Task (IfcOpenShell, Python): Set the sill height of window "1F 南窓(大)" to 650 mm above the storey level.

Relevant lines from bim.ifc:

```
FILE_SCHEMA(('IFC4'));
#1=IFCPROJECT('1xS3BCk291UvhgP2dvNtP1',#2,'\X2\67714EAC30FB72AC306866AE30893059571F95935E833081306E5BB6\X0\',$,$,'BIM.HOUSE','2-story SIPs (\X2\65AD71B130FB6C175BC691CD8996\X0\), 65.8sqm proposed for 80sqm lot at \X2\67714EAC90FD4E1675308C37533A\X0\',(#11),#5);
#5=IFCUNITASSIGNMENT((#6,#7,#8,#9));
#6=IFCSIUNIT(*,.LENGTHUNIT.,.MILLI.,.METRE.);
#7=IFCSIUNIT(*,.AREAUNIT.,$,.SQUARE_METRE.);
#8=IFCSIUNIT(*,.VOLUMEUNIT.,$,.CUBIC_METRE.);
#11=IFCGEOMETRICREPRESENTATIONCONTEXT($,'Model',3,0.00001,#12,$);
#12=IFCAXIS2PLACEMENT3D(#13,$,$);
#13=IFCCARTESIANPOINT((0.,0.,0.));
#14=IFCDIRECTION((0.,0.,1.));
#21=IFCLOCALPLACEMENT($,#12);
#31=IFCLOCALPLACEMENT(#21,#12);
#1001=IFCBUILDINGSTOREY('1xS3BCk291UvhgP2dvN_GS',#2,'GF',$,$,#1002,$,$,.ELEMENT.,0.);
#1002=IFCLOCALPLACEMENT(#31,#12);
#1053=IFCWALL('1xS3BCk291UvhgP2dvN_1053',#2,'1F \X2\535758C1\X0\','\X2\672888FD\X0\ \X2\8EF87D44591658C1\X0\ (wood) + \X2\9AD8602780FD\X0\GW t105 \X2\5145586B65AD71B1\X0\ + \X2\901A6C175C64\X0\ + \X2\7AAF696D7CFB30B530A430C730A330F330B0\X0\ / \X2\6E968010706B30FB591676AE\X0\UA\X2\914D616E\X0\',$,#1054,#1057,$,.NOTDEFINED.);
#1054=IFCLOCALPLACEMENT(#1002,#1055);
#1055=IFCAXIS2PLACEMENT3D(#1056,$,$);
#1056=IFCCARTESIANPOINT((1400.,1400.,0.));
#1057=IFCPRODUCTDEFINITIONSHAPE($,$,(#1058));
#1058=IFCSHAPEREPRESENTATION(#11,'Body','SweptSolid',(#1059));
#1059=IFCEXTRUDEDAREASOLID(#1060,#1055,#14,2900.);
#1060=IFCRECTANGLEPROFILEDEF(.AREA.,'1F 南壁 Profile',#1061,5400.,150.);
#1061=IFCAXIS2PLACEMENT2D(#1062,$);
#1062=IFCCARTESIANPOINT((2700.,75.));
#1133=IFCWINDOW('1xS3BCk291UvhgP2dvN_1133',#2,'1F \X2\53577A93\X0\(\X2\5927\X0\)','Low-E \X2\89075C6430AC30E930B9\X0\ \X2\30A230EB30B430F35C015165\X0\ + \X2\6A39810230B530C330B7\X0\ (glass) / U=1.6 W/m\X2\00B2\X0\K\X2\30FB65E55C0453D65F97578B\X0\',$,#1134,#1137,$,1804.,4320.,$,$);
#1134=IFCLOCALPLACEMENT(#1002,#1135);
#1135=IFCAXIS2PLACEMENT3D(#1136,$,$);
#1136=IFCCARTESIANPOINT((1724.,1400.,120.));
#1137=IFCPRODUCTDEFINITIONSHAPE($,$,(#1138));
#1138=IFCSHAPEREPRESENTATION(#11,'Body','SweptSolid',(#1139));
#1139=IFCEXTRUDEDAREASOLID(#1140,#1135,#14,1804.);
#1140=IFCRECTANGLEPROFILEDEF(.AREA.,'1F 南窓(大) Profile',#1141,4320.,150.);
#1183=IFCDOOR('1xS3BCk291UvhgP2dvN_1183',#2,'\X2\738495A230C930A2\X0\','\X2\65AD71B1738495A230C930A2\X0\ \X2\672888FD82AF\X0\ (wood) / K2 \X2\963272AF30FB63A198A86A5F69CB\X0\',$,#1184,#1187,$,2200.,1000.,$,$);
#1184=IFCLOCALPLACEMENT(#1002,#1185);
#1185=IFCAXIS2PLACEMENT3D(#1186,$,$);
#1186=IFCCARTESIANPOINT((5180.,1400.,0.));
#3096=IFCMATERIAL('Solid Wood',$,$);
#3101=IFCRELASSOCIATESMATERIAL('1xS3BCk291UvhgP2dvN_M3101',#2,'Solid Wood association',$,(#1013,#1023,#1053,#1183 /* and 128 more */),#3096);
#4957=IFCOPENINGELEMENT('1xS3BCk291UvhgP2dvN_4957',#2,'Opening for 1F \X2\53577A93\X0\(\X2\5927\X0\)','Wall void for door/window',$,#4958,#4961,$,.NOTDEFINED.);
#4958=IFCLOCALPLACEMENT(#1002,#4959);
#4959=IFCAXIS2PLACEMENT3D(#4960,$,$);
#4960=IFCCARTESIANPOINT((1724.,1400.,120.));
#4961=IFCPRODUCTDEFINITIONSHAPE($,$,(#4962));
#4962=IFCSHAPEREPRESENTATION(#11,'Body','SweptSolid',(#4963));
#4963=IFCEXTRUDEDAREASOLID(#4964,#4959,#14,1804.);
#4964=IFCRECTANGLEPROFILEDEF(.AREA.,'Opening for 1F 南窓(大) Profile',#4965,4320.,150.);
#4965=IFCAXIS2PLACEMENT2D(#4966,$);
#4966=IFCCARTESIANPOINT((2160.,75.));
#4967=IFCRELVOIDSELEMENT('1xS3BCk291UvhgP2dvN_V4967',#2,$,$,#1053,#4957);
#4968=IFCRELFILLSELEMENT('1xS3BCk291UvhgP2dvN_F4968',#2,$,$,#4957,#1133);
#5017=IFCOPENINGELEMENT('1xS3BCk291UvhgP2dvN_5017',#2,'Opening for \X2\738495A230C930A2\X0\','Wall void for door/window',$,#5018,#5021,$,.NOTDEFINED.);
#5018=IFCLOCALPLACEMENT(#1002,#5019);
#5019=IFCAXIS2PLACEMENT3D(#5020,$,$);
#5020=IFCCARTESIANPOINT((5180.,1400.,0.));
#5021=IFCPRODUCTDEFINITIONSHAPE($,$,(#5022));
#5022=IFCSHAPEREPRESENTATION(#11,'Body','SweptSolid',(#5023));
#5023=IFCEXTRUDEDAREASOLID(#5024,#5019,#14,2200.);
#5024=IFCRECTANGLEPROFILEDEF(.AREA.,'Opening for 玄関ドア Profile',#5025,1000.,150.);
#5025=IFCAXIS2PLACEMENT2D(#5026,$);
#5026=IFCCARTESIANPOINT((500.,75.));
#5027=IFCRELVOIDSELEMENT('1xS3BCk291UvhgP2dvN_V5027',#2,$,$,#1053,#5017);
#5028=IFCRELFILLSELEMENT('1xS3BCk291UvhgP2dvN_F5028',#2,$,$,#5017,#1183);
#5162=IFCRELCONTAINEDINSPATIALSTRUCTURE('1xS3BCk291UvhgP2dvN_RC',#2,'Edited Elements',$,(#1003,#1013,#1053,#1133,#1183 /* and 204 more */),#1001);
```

```python
import numpy as np
import ifcopenshell
import ifcopenshell.api.geometry
import ifcopenshell.geom
import ifcopenshell.util.element
import ifcopenshell.util.placement
import ifcopenshell.util.shape
import ifcopenshell.util.unit

model = ifcopenshell.open("bim.ifc")
unit_scale = ifcopenshell.util.unit.calculate_unit_scale(model)

window = model.by_id(1133)
opening = window.FillsVoids[0].RelatingOpeningElement
storey = ifcopenshell.util.element.get_container(window, ifc_class="IfcBuildingStorey")
level = ifcopenshell.util.placement.get_local_placement(storey.ObjectPlacement)[2, 3]

# The opening's origin need not be at the sill, so measure its lowest point.
shape = ifcopenshell.geom.create_shape(ifcopenshell.geom.settings(), opening)
bottom = ifcopenshell.util.shape.get_shape_bottom_elevation(shape, shape.geometry) / unit_scale
dz = level + 0.65 / unit_scale - bottom

shift = np.array([0.0, 0.0, dz])
# The window is not placed relative to its opening, so move both.
for product in (opening, window):
    matrix = ifcopenshell.util.placement.get_local_placement(product.ObjectPlacement)
    matrix[:3, 3] += shift
    ifcopenshell.api.geometry.edit_object_placement(model, product=product, matrix=matrix, is_si=False)

print(f"moved by {dz * unit_scale:+.3f} m")

model.write("bim_v2.ifc")
```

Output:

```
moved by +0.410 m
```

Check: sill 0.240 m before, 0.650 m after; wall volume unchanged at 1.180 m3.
